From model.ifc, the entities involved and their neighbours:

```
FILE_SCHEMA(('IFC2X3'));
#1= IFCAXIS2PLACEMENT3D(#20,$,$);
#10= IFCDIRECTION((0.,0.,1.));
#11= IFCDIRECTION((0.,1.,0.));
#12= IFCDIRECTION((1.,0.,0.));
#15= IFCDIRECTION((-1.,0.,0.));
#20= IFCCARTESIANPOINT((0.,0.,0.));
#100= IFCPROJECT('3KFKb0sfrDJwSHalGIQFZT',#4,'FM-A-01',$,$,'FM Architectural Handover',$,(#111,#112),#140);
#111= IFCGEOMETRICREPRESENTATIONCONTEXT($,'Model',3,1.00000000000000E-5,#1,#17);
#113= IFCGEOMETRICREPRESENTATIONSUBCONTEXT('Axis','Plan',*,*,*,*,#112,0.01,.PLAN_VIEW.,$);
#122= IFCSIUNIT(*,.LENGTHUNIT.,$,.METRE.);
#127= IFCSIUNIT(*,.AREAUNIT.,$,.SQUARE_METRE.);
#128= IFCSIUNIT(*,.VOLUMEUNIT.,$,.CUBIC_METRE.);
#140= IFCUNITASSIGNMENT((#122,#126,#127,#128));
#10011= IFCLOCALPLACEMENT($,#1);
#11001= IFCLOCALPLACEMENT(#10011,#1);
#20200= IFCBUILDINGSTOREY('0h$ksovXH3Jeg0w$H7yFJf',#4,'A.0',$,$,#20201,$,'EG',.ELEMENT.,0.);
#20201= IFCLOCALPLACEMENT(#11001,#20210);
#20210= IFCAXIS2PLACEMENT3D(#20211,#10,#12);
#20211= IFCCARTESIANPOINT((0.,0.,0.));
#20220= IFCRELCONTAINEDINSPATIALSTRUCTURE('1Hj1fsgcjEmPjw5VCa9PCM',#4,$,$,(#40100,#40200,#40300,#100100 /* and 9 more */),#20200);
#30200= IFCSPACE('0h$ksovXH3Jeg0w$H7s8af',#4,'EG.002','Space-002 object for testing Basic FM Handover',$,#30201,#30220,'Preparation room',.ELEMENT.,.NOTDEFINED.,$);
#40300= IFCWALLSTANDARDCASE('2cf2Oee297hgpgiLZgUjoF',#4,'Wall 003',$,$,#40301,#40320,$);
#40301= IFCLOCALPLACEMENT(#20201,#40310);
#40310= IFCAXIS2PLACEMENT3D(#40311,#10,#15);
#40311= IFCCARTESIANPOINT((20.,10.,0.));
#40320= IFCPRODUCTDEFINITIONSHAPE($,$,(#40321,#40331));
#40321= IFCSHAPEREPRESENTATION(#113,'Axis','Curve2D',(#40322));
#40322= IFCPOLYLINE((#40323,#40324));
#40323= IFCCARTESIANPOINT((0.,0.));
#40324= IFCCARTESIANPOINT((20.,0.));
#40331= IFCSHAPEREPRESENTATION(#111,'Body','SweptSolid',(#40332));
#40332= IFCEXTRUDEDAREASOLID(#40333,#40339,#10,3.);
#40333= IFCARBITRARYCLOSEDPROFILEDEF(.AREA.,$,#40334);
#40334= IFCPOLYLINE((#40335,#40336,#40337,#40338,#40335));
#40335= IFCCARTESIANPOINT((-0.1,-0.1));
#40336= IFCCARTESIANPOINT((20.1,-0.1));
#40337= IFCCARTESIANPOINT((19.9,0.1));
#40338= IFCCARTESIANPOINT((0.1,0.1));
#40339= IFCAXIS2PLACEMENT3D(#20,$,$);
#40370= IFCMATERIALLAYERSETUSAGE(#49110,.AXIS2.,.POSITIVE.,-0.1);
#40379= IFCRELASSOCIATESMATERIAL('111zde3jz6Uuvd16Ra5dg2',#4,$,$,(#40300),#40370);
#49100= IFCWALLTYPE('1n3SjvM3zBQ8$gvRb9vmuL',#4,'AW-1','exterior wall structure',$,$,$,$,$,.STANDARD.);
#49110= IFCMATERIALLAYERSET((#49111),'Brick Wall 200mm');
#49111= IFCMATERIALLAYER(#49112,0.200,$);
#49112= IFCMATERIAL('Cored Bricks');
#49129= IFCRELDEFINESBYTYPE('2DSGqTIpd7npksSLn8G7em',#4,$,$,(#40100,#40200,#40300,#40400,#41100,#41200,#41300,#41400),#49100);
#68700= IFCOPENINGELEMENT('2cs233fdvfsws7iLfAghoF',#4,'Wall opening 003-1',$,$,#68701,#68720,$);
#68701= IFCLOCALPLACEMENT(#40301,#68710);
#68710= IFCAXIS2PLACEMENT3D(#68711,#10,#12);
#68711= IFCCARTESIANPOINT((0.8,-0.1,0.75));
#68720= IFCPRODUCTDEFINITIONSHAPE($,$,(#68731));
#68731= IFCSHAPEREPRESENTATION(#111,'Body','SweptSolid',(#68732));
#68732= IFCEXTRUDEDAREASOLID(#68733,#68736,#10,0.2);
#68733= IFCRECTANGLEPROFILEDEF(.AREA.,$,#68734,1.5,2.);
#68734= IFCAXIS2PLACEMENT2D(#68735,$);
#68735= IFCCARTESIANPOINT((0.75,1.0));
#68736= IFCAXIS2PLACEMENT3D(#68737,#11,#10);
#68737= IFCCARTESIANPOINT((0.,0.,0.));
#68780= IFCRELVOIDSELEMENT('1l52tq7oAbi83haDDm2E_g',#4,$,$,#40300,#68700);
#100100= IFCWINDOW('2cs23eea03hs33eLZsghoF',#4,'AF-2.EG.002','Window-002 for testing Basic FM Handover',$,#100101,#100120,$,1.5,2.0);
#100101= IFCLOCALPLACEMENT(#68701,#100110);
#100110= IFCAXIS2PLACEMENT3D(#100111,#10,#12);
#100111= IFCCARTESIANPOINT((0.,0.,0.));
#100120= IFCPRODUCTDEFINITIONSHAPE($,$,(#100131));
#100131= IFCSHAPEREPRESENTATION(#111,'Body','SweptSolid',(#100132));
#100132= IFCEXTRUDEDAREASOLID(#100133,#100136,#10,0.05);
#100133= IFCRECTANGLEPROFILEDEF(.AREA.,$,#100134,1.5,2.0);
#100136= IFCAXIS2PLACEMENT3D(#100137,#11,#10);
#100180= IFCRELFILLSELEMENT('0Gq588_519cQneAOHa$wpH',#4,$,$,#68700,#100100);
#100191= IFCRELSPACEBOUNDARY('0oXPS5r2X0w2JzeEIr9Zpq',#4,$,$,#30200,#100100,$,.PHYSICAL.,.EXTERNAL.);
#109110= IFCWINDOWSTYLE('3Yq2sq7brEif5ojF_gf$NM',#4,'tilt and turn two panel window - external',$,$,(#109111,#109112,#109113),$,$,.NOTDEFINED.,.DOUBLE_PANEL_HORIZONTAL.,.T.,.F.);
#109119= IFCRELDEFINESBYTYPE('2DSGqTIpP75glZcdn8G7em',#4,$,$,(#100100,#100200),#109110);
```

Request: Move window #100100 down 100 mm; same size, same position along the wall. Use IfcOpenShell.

```python
import numpy as np
import ifcopenshell
import ifcopenshell.api.geometry
import ifcopenshell.util.placement
import ifcopenshell.util.unit

model = ifcopenshell.open("model.ifc")
unit_scale = ifcopenshell.util.unit.calculate_unit_scale(model)

window = model.by_id(100100)
opening = window.FillsVoids[0].RelatingOpeningElement
dz = -0.1 / unit_scale

shift = np.array([0.0, 0.0, dz])
# The window is placed relative to its opening, so it follows when the opening moves.
matrix = ifcopenshell.util.placement.get_local_placement(opening.ObjectPlacement)
matrix[:3, 3] += shift
ifcopenshell.api.geometry.edit_object_placement(
    model, product=opening, matrix=matrix, is_si=False, should_transform_children=True
)

print(f"moved by {dz * unit_scale:+.3f} m")

model.write("model-out.ifc")
```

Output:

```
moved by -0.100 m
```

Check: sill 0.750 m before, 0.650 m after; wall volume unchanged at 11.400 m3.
